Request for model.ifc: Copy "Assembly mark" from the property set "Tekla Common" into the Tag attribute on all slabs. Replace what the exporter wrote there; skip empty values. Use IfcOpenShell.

First a look at what the model holds.

```python
import ifcopenshell
import ifcopenshell.util.element

model = ifcopenshell.open("model.ifc")
print(model.schema)
slabs = model.by_type("IfcSlab")
print(len(slabs), "slabs")
for e in slabs[:8]:
    source = ifcopenshell.util.element.get_pset(e, "Tekla Common", "Assembly mark")
    target = e.Tag
    print(e.id(), repr(source), repr(target), sep=" | ")
```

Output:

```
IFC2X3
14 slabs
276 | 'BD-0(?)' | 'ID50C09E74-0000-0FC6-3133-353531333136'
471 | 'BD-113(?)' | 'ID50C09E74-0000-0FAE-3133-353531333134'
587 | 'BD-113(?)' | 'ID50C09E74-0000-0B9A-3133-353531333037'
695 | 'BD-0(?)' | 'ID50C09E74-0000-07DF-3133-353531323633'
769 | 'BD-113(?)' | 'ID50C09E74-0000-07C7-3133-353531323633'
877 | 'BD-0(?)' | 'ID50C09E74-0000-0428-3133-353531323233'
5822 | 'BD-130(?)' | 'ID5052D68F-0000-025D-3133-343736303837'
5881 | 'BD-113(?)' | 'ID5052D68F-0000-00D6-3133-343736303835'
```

```python
import ifcopenshell
import ifcopenshell.util.element

model = ifcopenshell.open("model.ifc")

count = 0
for e in model.by_type("IfcSlab"):
    value = ifcopenshell.util.element.get_pset(e, "Tekla Common", "Assembly mark")
    current = e.Tag
    if not value or not value.strip() or current == value:
        continue
    e.Tag = value
    count += 1

print(count, "slabs updated")

model.write("model_rev.ifc")
```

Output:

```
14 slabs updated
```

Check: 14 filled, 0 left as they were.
